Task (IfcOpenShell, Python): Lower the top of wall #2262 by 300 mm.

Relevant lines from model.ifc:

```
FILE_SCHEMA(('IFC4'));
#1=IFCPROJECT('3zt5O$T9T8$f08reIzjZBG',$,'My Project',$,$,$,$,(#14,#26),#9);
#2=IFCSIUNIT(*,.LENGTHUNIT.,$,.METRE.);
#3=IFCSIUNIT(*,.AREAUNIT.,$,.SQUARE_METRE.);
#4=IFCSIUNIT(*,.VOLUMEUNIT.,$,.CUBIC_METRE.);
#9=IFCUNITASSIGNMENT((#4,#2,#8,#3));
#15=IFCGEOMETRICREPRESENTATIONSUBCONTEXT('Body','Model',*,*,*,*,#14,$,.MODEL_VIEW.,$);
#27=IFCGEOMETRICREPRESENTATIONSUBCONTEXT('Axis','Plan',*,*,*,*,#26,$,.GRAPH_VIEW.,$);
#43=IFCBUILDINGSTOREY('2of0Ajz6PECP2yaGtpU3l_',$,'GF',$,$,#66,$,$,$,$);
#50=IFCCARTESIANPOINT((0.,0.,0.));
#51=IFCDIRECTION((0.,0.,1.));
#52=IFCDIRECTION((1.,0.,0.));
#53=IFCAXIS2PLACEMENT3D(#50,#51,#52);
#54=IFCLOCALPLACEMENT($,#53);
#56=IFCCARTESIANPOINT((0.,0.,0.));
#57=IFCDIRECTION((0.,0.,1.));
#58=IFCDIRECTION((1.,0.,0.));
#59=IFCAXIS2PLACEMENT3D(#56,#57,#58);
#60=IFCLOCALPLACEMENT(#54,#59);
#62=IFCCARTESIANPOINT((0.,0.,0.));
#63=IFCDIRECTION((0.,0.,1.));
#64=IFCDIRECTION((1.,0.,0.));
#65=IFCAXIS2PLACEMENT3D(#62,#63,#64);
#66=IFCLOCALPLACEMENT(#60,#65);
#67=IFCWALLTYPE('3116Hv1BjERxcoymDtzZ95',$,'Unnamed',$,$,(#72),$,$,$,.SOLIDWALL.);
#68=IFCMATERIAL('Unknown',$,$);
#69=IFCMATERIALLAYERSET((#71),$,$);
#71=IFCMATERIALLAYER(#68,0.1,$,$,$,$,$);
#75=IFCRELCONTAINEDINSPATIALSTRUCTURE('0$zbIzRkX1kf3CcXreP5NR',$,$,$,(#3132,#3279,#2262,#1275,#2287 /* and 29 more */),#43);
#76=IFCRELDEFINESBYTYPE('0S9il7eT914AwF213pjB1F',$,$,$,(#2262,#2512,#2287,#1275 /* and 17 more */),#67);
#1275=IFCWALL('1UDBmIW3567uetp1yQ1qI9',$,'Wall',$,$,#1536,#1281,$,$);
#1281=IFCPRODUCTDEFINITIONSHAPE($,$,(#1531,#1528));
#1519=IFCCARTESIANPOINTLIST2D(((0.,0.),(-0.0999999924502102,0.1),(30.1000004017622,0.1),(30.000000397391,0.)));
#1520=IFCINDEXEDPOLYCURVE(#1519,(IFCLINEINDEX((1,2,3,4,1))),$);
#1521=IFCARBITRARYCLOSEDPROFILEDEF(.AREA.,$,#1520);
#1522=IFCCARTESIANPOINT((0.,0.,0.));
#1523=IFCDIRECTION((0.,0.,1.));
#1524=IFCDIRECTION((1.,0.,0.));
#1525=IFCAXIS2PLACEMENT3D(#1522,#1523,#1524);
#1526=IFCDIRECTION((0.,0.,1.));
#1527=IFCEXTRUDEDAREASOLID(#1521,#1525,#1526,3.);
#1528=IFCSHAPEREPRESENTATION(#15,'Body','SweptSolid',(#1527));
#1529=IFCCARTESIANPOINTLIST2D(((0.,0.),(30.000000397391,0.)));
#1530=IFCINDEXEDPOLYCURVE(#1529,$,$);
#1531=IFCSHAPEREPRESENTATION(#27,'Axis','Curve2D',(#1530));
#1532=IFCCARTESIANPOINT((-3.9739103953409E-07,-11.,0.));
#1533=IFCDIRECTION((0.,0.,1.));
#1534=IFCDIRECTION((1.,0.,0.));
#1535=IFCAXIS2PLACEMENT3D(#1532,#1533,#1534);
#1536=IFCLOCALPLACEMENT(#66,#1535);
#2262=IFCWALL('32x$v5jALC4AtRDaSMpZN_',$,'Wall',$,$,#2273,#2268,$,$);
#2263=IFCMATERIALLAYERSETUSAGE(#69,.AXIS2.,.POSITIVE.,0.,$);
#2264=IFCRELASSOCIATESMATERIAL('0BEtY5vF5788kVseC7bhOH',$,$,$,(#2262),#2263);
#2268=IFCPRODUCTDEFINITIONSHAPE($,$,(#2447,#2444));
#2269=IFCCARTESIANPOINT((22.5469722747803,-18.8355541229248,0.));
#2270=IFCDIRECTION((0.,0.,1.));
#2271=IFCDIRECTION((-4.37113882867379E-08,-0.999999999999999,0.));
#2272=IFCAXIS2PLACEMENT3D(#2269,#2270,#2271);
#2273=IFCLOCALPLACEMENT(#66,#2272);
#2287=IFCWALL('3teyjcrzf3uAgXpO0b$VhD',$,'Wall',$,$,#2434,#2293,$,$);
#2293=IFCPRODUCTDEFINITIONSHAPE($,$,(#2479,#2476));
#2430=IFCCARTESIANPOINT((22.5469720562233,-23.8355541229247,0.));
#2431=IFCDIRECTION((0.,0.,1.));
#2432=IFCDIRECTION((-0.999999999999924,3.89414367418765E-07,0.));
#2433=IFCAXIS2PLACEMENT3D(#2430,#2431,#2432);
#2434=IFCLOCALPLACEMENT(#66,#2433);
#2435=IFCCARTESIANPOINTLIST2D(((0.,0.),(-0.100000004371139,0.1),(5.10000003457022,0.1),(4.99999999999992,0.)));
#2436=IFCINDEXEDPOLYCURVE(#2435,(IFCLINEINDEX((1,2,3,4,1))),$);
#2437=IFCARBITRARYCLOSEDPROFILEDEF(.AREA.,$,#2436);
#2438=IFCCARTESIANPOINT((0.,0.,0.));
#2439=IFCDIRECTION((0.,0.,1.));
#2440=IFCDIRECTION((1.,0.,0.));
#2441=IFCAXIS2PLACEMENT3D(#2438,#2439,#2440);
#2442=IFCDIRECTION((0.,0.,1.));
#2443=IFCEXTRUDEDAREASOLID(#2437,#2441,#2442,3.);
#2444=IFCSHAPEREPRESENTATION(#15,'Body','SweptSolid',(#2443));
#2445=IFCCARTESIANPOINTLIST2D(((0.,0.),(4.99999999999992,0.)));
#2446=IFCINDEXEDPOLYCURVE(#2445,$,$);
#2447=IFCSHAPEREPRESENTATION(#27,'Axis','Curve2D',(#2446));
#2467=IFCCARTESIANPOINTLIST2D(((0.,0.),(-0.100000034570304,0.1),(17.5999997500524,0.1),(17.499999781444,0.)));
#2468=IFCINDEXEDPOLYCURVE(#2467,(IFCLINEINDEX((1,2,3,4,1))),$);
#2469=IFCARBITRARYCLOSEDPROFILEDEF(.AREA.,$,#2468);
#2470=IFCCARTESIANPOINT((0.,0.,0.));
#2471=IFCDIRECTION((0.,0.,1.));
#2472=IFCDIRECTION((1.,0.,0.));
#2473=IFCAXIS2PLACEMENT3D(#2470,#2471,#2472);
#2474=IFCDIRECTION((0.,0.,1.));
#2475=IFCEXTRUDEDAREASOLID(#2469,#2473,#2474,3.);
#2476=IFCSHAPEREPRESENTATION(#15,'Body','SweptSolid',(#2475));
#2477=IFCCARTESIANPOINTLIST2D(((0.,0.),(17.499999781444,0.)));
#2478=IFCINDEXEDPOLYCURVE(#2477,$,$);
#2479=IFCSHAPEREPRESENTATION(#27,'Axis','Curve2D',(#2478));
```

```python
import ifcopenshell
import ifcopenshell.geom
import ifcopenshell.util.representation
import ifcopenshell.util.shape
import ifcopenshell.util.unit

model = ifcopenshell.open("model.ifc")
unit_scale = ifcopenshell.util.unit.calculate_unit_scale(model)
settings = ifcopenshell.geom.settings()


def volume(element):
    """Net volume in cubic metres, openings subtracted."""
    shape = ifcopenshell.geom.create_shape(settings, element)
    return ifcopenshell.util.shape.get_volume(shape.geometry)


wall = model.by_id(2262)
before = volume(wall)

body = ifcopenshell.util.representation.get_representation(wall, "Model", "Body")
solid = body.Items[0]
old_height = solid.Depth
solid.Depth -= 0.3 / unit_scale
after = volume(wall)

print(f"height {old_height:g} -> {solid.Depth:g}, volume {before:.3f} -> {after:.3f} m3")

model.write("model_v2.ifc")
```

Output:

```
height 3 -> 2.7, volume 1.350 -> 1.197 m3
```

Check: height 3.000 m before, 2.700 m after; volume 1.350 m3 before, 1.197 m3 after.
